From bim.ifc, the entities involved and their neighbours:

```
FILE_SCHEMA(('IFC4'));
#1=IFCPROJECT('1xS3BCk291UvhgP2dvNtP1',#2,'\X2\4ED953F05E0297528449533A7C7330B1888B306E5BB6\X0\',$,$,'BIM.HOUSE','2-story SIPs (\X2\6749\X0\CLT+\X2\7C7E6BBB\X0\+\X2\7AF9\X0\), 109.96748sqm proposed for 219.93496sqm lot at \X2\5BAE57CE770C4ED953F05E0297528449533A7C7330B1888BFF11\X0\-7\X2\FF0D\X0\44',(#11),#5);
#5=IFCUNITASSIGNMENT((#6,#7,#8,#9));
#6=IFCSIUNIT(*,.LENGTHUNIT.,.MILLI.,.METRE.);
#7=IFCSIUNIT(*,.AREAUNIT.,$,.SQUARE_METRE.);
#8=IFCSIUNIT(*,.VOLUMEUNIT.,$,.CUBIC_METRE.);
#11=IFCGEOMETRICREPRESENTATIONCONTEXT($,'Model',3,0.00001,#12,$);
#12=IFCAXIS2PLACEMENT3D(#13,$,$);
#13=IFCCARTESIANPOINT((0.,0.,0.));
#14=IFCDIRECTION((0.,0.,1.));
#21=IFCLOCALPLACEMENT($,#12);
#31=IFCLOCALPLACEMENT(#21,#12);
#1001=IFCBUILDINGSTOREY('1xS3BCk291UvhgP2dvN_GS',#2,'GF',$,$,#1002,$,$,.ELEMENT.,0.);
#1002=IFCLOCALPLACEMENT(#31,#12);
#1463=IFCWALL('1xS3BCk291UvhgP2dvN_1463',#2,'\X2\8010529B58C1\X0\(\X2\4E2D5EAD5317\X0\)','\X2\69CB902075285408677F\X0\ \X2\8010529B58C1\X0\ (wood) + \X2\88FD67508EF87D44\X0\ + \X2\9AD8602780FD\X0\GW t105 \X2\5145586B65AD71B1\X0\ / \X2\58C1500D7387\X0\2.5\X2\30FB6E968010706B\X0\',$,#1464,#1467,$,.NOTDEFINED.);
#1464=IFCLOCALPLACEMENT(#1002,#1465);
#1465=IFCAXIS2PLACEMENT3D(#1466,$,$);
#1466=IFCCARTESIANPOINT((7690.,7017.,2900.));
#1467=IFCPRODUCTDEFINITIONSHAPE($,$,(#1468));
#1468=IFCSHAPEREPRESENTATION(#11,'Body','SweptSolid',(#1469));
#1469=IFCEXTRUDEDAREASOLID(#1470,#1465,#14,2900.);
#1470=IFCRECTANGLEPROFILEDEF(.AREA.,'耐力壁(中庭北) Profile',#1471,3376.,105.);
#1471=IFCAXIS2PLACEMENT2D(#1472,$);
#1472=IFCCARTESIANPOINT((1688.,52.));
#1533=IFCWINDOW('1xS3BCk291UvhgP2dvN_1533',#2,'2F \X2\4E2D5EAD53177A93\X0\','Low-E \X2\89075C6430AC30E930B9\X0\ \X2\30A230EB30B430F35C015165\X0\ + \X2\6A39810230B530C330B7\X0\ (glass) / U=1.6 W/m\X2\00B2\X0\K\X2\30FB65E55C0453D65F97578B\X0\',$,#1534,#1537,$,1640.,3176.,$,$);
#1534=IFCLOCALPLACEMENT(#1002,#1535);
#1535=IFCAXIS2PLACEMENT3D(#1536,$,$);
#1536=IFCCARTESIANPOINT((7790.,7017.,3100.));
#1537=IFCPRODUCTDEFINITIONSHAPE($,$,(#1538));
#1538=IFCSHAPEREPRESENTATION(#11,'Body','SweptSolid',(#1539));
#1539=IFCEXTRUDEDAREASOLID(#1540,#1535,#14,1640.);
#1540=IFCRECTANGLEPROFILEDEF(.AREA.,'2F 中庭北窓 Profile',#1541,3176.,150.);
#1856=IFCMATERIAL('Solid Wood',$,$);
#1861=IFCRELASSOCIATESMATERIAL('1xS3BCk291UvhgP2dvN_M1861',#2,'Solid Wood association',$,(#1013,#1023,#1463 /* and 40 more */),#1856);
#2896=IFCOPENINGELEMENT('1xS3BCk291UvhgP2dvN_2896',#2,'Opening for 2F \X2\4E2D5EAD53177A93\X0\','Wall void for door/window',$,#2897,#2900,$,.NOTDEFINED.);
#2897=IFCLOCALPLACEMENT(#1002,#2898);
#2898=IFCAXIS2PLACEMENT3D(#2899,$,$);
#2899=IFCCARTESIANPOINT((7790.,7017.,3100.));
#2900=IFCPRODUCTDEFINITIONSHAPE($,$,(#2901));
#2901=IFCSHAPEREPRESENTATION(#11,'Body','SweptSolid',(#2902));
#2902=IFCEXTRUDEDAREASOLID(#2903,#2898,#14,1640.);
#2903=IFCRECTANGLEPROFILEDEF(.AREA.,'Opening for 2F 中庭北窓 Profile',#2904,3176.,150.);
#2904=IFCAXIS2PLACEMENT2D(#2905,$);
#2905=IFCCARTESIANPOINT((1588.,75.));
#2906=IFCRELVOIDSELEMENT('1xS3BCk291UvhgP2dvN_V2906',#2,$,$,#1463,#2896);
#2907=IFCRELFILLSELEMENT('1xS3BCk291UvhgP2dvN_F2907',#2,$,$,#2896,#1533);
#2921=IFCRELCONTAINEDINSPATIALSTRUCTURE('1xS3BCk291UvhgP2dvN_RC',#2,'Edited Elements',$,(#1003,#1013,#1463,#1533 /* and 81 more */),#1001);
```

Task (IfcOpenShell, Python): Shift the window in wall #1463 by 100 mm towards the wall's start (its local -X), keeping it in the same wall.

```python
import ifcopenshell
import ifcopenshell.api.geometry
import ifcopenshell.util.placement
import ifcopenshell.util.unit

model = ifcopenshell.open("bim.ifc")
unit_scale = ifcopenshell.util.unit.calculate_unit_scale(model)

window = model.by_guid("1xS3BCk291UvhgP2dvN_1533")
opening = window.FillsVoids[0].RelatingOpeningElement
wall = opening.VoidsElements[0].RelatingBuildingElement

wall_matrix = ifcopenshell.util.placement.get_local_placement(wall.ObjectPlacement)
shift = wall_matrix[:3, 0] * -0.1 / unit_scale
before = ifcopenshell.util.placement.get_local_placement(window.ObjectPlacement)[:3, 3].copy()

# The window is not placed relative to its opening, so move both.
for product in (opening, window):
    matrix = ifcopenshell.util.placement.get_local_placement(product.ObjectPlacement)
    matrix[:3, 3] += shift
    ifcopenshell.api.geometry.edit_object_placement(model, product=product, matrix=matrix, is_si=False)

after = ifcopenshell.util.placement.get_local_placement(window.ObjectPlacement)[:3, 3]
print("window moved by", (after - before).round(3) + 0.0)

model.write("bim-out.ifc")
```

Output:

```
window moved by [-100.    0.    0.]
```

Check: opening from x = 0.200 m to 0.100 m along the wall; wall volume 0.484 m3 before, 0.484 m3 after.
